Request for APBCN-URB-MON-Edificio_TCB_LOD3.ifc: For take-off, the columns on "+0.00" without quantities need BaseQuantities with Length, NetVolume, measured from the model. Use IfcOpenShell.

First a look at what the model holds.

```python
import ifcopenshell
import ifcopenshell.util.element
import ifcopenshell.util.unit

model = ifcopenshell.open("APBCN-URB-MON-Edificio_TCB_LOD3.ifc")
print(model.schema)
for unit_type in ("LENGTHUNIT", "AREAUNIT", "VOLUMEUNIT"):
    print(unit_type, ifcopenshell.util.unit.calculate_unit_scale(model, unit_type))
storey = next(s for s in model.by_type("IfcBuildingStorey") if s.Name == "+0.00")
columns = [e for e in ifcopenshell.util.element.get_decomposition(storey) if e.is_a("IfcColumn")]
for e in sorted(columns, key=lambda e: e.id()):
    print(e.id(), e.is_a(), e.Name, list(ifcopenshell.util.element.get_psets(e, qtos_only=True)), sep=" | ")
```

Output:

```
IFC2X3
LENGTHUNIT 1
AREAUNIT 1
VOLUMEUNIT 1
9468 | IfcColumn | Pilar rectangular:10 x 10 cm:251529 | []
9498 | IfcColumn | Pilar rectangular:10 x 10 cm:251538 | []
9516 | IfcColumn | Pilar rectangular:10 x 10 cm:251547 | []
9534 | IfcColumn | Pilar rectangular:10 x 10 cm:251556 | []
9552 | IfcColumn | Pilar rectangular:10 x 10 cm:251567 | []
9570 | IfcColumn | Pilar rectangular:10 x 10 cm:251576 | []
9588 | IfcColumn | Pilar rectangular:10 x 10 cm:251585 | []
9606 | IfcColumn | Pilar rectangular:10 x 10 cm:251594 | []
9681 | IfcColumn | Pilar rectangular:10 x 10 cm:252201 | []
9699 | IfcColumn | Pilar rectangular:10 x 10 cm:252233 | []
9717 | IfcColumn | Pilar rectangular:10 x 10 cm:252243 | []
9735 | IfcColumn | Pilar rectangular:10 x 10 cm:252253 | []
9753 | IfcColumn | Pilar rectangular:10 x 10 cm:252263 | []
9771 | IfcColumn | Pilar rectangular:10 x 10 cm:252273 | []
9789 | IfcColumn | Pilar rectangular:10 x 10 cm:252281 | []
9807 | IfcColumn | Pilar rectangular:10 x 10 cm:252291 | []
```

```python
import ifcopenshell
import ifcopenshell.api.pset
import ifcopenshell.geom
import ifcopenshell.util.element
import ifcopenshell.util.shape
import ifcopenshell.util.unit

model = ifcopenshell.open("APBCN-URB-MON-Edificio_TCB_LOD3.ifc")
unit_scale = ifcopenshell.util.unit.calculate_unit_scale(model)
volume_scale = ifcopenshell.util.unit.calculate_unit_scale(model, "VOLUMEUNIT")
settings = ifcopenshell.geom.settings()

storey = next(s for s in model.by_type("IfcBuildingStorey") if s.Name == "+0.00")
columns = [e for e in ifcopenshell.util.element.get_decomposition(storey) if e.is_a("IfcColumn")]

for e in sorted(columns, key=lambda e: e.id()):
    if ifcopenshell.util.element.get_psets(e, qtos_only=True, should_inherit=False):
        continue
    # Geometry comes back in metres, in the element's own axes.
    shape = ifcopenshell.geom.create_shape(settings, e)
    values = {
        "Length": ifcopenshell.util.shape.get_z(shape.geometry) / unit_scale,
        "NetVolume": ifcopenshell.util.shape.get_volume(shape.geometry) / volume_scale,
    }
    qto = ifcopenshell.api.pset.add_qto(model, product=e, name="BaseQuantities")
    ifcopenshell.api.pset.edit_qto(model, qto=qto, properties=values)
    print(e.id(), {k: round(v, 3) for k, v in values.items()})

model.write("APBCN-URB-MON-Edificio_TCB_LOD3_edited.ifc")
```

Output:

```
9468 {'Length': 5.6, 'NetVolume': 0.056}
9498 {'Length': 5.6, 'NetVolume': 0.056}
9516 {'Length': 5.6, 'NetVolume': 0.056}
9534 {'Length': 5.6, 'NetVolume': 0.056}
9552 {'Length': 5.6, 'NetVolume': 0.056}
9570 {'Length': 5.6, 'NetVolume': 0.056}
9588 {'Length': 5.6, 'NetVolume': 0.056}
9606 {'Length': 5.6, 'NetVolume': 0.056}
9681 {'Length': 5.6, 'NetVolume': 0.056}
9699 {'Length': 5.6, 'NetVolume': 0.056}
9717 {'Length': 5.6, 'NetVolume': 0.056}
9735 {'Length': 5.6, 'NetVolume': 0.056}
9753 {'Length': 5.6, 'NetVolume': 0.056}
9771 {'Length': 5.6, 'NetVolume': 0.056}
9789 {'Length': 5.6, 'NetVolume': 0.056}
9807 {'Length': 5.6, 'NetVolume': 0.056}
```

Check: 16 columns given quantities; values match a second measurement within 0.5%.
